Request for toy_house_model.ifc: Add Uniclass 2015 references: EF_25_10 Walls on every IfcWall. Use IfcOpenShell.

First a look at what the model holds.

```python
import ifcopenshell

model = ifcopenshell.open("toy_house_model.ifc")
print(model.schema)
print("classifications:", [c.Name for c in model.by_type("IfcClassification")])
for ifc_class in ("IfcDoor", "IfcRoof", "IfcStair", "IfcWall", "IfcWindow"):
    print(ifc_class, len(model.by_type(ifc_class)))
```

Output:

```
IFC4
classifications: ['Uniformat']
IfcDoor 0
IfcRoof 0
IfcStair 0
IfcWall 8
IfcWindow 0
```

```python
import ifcopenshell
import ifcopenshell.api.classification

model = ifcopenshell.open("toy_house_model.ifc")

system = ifcopenshell.api.classification.add_classification(model, classification="Uniclass 2015")

codes = {
    "IfcWall": ("EF_25_10", "Walls"),
}
for ifc_class, (code, name) in codes.items():
    products = model.by_type(ifc_class)
    ifcopenshell.api.classification.add_reference(
        model, products=products, classification=system, identification=code, name=name
    )
    print(code, len(products))

model.write("toy_house_model_v2.ifc")
```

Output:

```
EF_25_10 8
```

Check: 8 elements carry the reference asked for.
